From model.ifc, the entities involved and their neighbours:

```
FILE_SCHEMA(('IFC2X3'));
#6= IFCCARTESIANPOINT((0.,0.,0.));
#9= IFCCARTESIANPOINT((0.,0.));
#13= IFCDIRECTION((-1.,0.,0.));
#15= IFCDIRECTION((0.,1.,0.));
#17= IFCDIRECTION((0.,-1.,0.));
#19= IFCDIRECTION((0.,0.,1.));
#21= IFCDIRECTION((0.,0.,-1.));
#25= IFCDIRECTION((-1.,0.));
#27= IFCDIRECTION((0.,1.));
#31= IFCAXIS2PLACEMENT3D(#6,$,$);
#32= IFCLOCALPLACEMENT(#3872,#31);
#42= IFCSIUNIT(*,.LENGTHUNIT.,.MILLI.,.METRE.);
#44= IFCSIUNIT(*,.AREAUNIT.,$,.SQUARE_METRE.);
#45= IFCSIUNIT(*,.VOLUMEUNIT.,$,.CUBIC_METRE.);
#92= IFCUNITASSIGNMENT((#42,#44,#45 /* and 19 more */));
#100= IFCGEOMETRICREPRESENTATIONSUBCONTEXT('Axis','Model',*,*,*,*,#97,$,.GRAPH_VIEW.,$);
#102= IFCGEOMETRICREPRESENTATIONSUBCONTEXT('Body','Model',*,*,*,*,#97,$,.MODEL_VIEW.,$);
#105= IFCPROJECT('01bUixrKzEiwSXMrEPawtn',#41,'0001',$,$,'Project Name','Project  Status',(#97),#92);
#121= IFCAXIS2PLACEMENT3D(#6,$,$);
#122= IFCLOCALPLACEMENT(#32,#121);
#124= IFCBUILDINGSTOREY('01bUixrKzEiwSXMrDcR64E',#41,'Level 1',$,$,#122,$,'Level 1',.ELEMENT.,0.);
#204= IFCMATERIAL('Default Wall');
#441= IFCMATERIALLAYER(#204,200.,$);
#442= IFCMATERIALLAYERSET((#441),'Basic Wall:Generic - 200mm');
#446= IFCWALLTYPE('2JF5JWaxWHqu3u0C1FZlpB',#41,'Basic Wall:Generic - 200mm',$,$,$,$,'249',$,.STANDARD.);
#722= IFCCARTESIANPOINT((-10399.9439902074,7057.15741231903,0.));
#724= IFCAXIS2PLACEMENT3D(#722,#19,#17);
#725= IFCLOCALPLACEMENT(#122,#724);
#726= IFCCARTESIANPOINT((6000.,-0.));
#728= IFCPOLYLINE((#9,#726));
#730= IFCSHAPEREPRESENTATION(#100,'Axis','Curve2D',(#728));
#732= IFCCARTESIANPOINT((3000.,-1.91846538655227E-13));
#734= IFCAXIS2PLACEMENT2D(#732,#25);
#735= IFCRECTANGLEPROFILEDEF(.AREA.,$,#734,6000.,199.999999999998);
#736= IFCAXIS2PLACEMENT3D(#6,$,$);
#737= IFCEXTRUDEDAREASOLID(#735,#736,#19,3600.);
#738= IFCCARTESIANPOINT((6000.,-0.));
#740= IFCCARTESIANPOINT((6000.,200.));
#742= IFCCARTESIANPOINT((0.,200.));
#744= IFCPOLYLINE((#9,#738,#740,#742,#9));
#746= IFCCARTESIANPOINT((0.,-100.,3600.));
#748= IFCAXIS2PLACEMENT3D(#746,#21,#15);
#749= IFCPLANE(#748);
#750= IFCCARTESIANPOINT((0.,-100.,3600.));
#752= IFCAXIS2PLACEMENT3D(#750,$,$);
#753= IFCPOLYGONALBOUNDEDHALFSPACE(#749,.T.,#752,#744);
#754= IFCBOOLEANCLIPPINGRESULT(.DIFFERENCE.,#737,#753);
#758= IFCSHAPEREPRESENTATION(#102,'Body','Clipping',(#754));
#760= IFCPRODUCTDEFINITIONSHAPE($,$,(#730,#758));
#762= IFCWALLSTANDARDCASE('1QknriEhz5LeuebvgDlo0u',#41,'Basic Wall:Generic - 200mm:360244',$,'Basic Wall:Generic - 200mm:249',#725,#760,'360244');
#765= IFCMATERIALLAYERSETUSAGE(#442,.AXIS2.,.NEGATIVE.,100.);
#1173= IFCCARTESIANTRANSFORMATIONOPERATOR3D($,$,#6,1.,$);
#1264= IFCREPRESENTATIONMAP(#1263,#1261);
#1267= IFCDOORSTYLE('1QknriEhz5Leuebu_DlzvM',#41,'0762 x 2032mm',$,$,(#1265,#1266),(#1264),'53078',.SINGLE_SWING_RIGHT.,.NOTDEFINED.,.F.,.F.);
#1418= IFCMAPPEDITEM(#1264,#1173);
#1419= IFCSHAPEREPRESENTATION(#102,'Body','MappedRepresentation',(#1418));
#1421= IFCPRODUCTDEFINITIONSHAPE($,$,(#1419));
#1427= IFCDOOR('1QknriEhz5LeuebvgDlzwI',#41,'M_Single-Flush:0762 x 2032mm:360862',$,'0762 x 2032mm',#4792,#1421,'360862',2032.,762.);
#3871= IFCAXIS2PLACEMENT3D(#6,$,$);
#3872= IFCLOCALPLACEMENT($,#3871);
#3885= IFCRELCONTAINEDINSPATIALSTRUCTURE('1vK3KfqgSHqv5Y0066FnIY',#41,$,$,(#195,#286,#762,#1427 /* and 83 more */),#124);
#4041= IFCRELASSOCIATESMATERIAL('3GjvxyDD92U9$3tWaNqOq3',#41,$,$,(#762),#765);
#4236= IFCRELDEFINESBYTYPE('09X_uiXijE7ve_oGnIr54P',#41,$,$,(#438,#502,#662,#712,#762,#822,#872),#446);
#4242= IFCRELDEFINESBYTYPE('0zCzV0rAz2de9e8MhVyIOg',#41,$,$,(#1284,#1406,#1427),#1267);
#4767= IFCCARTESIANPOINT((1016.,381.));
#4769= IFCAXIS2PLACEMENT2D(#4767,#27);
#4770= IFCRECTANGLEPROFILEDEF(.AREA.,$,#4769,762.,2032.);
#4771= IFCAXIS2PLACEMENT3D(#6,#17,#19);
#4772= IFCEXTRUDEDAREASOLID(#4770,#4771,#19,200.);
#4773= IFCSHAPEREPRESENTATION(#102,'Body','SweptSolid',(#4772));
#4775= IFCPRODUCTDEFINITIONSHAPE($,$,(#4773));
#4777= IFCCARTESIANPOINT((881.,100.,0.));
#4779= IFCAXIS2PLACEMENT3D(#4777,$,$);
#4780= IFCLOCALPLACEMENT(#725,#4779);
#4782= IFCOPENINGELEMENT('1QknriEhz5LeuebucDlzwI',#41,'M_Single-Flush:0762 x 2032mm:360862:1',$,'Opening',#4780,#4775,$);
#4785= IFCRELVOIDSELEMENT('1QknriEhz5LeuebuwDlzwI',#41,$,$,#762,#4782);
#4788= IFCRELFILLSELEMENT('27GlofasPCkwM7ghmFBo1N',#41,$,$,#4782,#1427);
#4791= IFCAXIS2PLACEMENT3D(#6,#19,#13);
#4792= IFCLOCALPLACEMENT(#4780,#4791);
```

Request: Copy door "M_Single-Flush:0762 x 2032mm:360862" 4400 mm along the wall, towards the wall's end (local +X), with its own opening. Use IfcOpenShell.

```python
import ifcopenshell
import ifcopenshell.api.feature
import ifcopenshell.api.geometry
import ifcopenshell.api.root
import ifcopenshell.geom
import ifcopenshell.util.element
import ifcopenshell.util.placement
import ifcopenshell.util.shape

model = ifcopenshell.open("model.ifc")
settings = ifcopenshell.geom.settings()


def volume(element):
    """Net volume in cubic metres, openings subtracted."""
    shape = ifcopenshell.geom.create_shape(settings, element)
    return ifcopenshell.util.shape.get_volume(shape.geometry)


def reuse_history(source, copy):
    """copy_class also copies each property set's owner history, people and application; keep the originals."""
    for rel in copy.IsDefinedBy:
        if rel.is_a("IfcRelDefinesByProperties") and (history := rel.RelatingPropertyDefinition.OwnerHistory):
            rel.RelatingPropertyDefinition.OwnerHistory = source.OwnerHistory
            ifcopenshell.util.element.remove_deep2(model, history)


door = model.by_guid("1QknriEhz5LeuebvgDlzwI")
opening = door.FillsVoids[0].RelatingOpeningElement
wall = opening.VoidsElements[0].RelatingBuildingElement
before = volume(wall)
shift = ifcopenshell.util.placement.get_local_placement(wall.ObjectPlacement)[:3, 0] * 4400.0

# copy_class copies the void relationship, type, container and properties, but no geometry.
new_opening = ifcopenshell.api.root.copy_class(model, product=opening)
new_opening.Representation = ifcopenshell.util.element.copy_deep(
    model, opening.Representation, exclude=["IfcGeometricRepresentationContext", "IfcRepresentationMap"]
)
new_opening.Name = "M_Single-Flush:0762 x 2032mm"
new_door = ifcopenshell.api.root.copy_class(model, product=door)
new_door.Representation = ifcopenshell.util.element.copy_deep(
    model, door.Representation, exclude=["IfcGeometricRepresentationContext", "IfcRepresentationMap"]
)
new_door.Name = "M_Single-Flush:0762 x 2032mm"
new_door.Tag = None
reuse_history(door, new_door)
fills = ifcopenshell.api.feature.add_filling(model, opening=new_opening, element=new_door)
fills.OwnerHistory = new_door.OwnerHistory  # required in IFC2X3

for old, new in ((opening, new_opening), (door, new_door)):
    matrix = ifcopenshell.util.placement.get_local_placement(old.ObjectPlacement)
    matrix[:3, 3] += shift
    ifcopenshell.api.geometry.edit_object_placement(model, product=new, matrix=matrix, is_si=False)

after = volume(wall)

print(f"wall volume {before:.3f} -> {after:.3f} m3")

model.write("model_v2.ifc")
```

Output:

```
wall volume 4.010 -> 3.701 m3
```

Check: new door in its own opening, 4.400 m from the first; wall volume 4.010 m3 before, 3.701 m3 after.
